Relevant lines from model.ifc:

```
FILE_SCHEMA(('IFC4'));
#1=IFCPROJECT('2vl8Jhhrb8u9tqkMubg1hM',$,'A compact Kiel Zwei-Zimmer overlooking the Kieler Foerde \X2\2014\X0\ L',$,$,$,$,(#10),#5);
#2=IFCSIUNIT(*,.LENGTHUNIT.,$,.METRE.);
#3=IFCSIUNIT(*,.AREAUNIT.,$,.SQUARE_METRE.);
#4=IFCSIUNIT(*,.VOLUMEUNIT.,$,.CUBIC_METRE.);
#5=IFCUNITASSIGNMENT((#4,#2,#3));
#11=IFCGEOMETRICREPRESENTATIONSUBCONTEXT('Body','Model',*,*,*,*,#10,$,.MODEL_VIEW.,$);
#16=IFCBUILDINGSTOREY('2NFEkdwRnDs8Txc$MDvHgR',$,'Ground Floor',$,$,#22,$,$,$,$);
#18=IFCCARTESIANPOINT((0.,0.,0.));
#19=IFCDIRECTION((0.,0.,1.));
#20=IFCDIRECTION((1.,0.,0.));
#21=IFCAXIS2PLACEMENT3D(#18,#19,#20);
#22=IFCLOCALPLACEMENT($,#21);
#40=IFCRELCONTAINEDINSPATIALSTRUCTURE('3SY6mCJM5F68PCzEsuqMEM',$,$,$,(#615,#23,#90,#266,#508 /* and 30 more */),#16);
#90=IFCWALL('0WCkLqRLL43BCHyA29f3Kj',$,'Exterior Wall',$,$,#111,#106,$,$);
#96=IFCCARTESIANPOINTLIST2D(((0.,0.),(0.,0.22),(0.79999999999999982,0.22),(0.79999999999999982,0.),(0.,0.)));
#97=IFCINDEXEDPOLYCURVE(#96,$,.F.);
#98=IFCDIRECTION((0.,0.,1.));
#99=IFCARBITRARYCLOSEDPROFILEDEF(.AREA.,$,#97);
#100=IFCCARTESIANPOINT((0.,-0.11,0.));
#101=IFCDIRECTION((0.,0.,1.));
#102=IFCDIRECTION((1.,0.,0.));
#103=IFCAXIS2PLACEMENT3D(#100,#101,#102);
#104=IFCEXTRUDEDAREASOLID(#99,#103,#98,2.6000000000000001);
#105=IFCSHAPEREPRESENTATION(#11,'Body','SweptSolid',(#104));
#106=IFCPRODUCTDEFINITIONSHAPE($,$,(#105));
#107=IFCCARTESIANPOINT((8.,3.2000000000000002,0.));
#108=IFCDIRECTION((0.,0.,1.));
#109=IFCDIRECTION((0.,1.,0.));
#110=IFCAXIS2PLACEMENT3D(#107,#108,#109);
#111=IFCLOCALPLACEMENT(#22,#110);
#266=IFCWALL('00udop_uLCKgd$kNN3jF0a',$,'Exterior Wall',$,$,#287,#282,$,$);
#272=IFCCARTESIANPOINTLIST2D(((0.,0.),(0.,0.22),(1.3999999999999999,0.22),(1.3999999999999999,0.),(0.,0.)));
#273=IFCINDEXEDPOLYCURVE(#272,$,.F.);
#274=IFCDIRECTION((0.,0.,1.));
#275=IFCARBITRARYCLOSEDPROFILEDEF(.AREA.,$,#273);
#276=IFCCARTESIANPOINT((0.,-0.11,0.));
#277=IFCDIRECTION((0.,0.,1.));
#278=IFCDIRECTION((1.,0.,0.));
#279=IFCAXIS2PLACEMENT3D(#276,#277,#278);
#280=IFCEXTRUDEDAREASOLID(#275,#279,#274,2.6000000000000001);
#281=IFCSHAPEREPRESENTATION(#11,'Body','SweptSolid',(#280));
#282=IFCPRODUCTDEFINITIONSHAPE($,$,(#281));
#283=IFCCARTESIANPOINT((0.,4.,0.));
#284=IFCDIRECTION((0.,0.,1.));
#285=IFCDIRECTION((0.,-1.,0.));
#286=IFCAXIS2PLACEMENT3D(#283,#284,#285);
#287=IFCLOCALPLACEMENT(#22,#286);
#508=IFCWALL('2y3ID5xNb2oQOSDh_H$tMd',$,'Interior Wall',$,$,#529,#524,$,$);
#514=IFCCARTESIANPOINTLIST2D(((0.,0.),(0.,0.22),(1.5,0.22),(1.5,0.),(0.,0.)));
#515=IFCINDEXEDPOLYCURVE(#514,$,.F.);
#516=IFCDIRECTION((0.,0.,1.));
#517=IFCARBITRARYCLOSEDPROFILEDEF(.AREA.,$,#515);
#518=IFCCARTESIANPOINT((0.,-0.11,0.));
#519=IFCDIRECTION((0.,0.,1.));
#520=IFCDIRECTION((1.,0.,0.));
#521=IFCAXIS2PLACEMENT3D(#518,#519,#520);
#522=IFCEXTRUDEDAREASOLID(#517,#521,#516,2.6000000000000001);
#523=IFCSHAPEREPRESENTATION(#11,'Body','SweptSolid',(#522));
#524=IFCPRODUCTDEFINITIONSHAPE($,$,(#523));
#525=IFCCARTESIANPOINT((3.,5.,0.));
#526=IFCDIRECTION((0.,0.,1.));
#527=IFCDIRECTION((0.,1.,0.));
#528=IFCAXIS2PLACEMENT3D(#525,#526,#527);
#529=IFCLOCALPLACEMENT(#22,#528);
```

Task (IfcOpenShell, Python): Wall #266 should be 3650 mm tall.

```python
import ifcopenshell
import ifcopenshell.geom
import ifcopenshell.util.representation
import ifcopenshell.util.shape

model = ifcopenshell.open("model.ifc")
settings = ifcopenshell.geom.settings()


def volume(element):
    """Net volume in cubic metres, openings subtracted."""
    shape = ifcopenshell.geom.create_shape(settings, element)
    return ifcopenshell.util.shape.get_volume(shape.geometry)


wall = model.by_guid("00udop_uLCKgd$kNN3jF0a")
before = volume(wall)

body = ifcopenshell.util.representation.get_representation(wall, "Model", "Body")
solid = body.Items[0]
old_height = solid.Depth
solid.Depth = 3.65
after = volume(wall)

print(f"height {old_height:g} -> {solid.Depth:g}, volume {before:.3f} -> {after:.3f} m3")

model.write("model_rev.ifc")
```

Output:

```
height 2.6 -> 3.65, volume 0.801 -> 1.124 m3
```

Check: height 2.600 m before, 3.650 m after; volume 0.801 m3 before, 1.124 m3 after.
